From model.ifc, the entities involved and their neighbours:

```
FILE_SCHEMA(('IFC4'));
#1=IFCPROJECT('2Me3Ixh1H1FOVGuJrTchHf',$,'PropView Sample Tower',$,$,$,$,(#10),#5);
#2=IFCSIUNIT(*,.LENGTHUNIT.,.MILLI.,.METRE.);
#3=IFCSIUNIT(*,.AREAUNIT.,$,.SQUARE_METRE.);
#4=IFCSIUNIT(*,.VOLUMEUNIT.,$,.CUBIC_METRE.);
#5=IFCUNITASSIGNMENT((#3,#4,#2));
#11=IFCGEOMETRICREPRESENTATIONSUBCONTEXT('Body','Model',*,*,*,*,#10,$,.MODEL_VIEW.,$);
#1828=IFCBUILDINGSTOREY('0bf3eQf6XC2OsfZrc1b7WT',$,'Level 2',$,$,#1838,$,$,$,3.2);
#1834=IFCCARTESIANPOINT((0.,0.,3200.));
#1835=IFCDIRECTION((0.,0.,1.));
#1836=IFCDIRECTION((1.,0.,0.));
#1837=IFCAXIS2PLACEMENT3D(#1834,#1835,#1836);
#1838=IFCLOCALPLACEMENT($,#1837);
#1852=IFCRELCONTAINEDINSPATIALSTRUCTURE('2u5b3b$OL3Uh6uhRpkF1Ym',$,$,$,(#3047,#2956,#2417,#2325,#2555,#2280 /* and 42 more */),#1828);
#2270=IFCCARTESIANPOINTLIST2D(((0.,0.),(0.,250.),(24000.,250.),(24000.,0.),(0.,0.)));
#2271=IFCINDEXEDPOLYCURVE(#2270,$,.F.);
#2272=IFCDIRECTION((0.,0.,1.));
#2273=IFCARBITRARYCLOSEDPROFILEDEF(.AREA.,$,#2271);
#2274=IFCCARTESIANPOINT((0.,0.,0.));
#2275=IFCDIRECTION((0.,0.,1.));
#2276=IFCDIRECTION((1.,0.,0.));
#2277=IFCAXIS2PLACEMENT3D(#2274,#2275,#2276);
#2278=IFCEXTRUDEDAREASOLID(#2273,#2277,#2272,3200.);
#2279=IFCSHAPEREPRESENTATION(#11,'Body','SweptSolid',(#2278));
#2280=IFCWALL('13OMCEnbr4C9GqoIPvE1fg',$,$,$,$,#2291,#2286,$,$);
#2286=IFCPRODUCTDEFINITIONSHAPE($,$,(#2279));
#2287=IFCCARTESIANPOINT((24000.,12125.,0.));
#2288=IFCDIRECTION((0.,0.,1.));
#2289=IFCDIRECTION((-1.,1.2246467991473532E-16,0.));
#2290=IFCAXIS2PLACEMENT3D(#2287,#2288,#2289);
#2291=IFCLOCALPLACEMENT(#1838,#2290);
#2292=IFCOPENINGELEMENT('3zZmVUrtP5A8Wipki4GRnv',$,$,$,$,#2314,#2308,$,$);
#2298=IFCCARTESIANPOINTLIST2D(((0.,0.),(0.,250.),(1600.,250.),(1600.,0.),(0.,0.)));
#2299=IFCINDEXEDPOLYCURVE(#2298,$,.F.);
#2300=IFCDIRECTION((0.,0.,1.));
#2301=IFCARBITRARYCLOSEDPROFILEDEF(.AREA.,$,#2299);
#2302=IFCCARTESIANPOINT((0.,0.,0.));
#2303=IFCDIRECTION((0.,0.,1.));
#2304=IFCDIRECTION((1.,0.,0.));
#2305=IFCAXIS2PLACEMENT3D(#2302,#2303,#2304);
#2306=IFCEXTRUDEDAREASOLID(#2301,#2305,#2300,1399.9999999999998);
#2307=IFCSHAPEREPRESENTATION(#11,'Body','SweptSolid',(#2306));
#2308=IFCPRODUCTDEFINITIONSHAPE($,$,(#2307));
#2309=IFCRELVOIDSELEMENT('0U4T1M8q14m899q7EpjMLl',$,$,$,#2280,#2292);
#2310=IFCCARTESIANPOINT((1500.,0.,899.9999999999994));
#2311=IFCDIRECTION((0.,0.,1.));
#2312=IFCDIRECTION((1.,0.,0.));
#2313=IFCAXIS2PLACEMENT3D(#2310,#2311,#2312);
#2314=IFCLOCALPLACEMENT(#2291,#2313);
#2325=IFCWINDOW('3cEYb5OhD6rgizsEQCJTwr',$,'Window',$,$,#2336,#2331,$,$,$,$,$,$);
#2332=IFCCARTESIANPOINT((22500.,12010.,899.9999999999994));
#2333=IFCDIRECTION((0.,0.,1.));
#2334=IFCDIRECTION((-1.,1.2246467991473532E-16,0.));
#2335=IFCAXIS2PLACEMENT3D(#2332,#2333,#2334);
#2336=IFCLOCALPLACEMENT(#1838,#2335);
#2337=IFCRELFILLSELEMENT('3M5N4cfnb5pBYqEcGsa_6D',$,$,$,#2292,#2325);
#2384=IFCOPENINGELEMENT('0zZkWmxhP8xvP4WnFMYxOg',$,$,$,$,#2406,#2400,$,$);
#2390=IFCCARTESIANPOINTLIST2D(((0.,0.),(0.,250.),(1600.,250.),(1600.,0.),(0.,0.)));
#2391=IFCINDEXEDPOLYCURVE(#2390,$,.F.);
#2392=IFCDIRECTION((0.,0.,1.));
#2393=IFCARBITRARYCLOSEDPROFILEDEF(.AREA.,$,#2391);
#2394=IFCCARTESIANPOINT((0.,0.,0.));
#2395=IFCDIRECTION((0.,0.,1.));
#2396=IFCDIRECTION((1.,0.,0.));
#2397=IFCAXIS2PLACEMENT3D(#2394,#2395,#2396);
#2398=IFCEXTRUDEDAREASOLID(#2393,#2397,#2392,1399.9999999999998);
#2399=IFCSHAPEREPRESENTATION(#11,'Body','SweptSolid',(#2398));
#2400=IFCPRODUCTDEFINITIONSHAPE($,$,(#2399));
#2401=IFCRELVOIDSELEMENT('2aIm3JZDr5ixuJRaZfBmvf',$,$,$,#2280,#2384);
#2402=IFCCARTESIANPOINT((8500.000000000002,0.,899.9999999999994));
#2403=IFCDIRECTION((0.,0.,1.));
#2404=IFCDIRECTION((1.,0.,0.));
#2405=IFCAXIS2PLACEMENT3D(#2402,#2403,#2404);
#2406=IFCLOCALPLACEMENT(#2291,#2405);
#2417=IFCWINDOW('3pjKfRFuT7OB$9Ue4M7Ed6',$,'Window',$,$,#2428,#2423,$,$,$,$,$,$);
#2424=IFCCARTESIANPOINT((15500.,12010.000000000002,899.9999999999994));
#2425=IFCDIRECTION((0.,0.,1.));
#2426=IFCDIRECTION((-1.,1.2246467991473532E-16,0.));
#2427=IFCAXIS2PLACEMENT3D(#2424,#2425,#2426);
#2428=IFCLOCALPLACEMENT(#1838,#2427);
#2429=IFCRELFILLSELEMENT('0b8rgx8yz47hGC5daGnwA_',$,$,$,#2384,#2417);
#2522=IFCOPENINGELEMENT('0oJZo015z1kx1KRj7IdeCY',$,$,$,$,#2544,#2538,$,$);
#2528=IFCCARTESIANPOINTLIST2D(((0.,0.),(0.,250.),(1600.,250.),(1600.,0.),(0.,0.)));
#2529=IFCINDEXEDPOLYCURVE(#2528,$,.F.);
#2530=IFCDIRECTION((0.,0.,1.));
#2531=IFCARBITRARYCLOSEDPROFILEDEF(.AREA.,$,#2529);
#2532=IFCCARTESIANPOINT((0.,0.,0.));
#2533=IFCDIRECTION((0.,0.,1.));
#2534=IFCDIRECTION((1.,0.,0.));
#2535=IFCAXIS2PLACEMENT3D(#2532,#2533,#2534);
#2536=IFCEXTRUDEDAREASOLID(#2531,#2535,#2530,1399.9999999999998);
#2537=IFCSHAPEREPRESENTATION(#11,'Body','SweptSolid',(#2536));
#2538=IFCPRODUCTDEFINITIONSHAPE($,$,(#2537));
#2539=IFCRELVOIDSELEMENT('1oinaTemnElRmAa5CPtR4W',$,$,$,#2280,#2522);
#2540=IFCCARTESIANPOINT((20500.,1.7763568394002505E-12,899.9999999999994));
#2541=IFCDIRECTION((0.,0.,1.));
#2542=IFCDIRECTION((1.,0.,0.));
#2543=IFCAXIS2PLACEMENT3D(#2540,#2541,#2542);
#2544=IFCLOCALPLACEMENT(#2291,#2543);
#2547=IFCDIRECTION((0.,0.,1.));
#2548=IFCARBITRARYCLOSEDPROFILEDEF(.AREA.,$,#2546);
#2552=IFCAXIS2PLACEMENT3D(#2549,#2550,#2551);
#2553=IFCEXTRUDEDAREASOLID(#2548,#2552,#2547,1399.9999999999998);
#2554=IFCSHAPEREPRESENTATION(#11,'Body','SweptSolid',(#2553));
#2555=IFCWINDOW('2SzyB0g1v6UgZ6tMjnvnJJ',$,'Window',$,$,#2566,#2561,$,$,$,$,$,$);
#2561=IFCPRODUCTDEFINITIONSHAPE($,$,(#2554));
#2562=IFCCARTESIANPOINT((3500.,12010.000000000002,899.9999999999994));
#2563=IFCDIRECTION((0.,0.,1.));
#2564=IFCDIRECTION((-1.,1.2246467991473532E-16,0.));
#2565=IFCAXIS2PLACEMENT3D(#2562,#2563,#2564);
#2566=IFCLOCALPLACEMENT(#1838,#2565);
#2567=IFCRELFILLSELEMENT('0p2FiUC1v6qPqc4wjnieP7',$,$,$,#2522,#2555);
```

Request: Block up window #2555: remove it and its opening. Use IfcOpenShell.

```python
import ifcopenshell
import ifcopenshell.api.feature
import ifcopenshell.api.root
import ifcopenshell.geom
import ifcopenshell.util.shape

model = ifcopenshell.open("model.ifc")
settings = ifcopenshell.geom.settings()


def volume(element):
    """Net volume in cubic metres, openings subtracted."""
    shape = ifcopenshell.geom.create_shape(settings, element)
    return ifcopenshell.util.shape.get_volume(shape.geometry)


window = model.by_guid("2SzyB0g1v6UgZ6tMjnvnJJ")
opening = window.FillsVoids[0].RelatingOpeningElement
wall = opening.VoidsElements[0].RelatingBuildingElement
before = volume(wall)

ifcopenshell.api.root.remove_product(model, product=window)
ifcopenshell.api.feature.remove_feature(model, feature=opening)

after = volume(wall)

print(f"wall volume {before:.3f} -> {after:.3f} m3")

model.write("model_edited.ifc")
```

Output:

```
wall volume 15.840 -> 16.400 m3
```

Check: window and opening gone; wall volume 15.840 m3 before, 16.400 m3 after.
